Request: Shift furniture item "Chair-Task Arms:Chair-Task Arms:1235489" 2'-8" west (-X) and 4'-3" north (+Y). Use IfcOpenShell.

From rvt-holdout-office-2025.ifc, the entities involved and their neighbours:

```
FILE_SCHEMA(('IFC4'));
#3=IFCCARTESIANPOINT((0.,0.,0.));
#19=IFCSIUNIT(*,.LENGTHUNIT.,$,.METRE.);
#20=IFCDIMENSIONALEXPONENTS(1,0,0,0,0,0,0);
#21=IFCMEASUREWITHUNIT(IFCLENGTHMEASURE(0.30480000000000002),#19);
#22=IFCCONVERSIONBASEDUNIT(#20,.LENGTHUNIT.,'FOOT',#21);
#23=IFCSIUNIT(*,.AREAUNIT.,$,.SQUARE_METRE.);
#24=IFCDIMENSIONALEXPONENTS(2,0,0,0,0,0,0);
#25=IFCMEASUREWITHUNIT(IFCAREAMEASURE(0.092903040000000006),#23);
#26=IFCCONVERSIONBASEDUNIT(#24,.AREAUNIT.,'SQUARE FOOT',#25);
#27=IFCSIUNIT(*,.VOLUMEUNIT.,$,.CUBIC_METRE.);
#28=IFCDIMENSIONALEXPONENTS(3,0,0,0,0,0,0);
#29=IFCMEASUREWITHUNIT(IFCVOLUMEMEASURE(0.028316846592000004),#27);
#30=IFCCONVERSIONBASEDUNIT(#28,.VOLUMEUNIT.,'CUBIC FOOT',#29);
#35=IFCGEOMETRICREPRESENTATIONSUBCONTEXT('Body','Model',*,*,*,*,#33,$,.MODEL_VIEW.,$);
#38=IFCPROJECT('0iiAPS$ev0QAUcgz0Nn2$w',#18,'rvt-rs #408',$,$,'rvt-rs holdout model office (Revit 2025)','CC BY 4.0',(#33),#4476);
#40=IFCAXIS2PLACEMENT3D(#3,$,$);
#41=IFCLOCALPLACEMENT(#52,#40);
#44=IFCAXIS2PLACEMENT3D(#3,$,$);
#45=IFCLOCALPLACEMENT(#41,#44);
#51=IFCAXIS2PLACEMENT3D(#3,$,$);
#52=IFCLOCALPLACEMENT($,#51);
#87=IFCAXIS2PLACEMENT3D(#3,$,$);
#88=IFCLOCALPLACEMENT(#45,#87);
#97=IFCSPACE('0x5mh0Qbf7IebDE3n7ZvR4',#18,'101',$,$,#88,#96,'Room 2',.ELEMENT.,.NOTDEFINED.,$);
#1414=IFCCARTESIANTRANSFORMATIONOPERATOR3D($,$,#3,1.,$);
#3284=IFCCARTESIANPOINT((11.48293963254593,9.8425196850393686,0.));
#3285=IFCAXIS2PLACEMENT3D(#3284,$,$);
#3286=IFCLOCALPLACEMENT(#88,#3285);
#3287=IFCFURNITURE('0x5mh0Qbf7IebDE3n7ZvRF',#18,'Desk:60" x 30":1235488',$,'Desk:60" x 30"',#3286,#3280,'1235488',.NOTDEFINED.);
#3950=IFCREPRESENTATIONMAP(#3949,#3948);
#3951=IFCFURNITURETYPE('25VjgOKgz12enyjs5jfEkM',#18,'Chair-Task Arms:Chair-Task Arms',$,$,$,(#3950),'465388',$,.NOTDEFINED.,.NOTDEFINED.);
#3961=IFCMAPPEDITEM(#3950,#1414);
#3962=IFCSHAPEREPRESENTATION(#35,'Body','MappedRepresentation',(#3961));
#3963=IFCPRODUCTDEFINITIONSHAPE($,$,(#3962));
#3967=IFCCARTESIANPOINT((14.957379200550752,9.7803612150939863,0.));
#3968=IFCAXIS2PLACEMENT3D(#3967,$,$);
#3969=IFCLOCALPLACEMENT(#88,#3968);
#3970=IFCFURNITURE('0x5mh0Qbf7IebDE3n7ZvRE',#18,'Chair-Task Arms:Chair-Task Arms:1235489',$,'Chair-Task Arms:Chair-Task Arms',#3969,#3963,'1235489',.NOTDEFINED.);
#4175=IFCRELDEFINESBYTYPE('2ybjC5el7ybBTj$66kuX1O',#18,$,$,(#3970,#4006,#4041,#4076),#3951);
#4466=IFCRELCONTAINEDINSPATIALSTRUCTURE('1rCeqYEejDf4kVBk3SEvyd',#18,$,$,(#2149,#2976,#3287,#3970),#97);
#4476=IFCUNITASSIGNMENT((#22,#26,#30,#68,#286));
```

```python
import ifcopenshell
import ifcopenshell.api.geometry
import ifcopenshell.util.placement
import ifcopenshell.util.unit

model = ifcopenshell.open("rvt-holdout-office-2025.ifc")
unit_scale = ifcopenshell.util.unit.calculate_unit_scale(model)

item = model.by_guid("0x5mh0Qbf7IebDE3n7ZvRE")
matrix = ifcopenshell.util.placement.get_local_placement(item.ObjectPlacement)
matrix[0, 3] -= 32 * 0.0254 / unit_scale
matrix[1, 3] += 51 * 0.0254 / unit_scale
ifcopenshell.api.geometry.edit_object_placement(model, product=item, matrix=matrix, is_si=False)

print(ifcopenshell.util.placement.get_local_placement(item.ObjectPlacement).round(3) + 0.0)

model.write("rvt-holdout-office-2025_v2.ifc")
```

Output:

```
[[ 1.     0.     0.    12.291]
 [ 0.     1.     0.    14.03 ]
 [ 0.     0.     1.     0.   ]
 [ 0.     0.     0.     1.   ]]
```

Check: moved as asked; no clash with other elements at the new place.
